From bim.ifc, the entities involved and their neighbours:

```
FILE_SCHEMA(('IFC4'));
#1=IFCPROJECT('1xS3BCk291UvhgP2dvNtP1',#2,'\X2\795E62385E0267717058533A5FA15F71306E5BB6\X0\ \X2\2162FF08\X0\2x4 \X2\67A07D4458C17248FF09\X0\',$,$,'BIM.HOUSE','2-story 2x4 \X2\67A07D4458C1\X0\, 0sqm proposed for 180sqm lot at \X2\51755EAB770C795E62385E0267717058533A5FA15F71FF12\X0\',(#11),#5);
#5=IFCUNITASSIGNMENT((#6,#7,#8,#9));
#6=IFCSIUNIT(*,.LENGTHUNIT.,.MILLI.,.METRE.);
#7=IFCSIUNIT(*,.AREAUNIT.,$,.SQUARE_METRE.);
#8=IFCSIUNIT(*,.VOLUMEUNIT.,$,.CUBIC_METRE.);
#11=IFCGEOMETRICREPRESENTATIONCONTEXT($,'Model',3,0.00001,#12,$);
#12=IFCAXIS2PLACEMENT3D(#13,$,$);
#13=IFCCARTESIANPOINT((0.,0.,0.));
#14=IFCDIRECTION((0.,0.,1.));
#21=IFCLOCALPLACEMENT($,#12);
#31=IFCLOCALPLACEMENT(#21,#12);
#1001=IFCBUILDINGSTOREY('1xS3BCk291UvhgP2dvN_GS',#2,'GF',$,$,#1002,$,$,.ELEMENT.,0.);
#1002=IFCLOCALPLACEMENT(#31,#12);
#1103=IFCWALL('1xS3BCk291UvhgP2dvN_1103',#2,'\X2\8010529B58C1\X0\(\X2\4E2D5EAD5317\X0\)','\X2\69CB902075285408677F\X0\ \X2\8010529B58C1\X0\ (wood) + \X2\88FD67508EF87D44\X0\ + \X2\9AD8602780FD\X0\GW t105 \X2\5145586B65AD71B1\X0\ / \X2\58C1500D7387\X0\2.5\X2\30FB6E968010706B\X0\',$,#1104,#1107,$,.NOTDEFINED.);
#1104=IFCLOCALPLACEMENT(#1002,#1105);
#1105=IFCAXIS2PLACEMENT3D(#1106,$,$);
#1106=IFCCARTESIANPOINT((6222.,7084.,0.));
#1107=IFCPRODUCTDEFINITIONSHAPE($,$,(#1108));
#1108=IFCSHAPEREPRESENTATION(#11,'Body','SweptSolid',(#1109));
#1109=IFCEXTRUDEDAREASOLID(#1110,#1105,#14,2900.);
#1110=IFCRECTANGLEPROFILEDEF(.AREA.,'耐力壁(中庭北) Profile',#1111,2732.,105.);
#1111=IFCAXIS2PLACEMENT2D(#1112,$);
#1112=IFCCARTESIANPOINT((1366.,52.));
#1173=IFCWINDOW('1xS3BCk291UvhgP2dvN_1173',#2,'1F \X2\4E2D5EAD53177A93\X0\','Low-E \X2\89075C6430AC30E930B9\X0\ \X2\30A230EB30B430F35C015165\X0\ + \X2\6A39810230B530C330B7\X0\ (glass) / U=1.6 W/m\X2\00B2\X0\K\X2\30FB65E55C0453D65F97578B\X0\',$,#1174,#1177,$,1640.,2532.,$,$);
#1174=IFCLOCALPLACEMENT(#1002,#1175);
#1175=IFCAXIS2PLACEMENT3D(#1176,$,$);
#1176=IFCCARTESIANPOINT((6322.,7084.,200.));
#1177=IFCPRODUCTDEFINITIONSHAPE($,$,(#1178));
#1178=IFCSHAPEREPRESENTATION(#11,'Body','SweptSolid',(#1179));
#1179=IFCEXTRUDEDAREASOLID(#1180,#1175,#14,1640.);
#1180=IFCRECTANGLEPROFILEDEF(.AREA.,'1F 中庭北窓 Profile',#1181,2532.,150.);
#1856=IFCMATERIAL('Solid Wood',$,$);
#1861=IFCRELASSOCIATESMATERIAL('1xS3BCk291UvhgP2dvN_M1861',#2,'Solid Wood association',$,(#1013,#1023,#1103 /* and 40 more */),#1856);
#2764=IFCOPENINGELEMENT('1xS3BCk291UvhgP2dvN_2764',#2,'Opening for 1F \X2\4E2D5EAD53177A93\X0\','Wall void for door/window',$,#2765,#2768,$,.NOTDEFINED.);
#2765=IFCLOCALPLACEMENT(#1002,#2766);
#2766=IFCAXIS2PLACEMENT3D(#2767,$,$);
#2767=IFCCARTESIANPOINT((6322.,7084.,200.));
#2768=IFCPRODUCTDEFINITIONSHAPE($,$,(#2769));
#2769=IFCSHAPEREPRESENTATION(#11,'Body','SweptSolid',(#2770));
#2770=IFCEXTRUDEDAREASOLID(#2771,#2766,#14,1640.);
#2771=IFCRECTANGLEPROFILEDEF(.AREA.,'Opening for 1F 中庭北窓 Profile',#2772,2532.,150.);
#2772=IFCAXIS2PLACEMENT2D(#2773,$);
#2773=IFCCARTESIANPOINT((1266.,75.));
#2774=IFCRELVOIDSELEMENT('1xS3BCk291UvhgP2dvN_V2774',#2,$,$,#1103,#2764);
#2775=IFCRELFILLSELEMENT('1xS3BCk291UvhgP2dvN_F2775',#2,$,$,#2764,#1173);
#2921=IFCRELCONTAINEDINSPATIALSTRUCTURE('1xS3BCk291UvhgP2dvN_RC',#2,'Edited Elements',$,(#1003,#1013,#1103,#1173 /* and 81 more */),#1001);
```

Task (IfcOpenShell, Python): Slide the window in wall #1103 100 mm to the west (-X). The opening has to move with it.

```python
import ifcopenshell
import ifcopenshell.api.geometry
import ifcopenshell.util.placement

model = ifcopenshell.open("bim.ifc")

window = model.by_guid("1xS3BCk291UvhgP2dvN_1173")
opening = window.FillsVoids[0].RelatingOpeningElement
wall = opening.VoidsElements[0].RelatingBuildingElement

wall_matrix = ifcopenshell.util.placement.get_local_placement(wall.ObjectPlacement)
shift = wall_matrix[:3, 0] * -100.0
before = ifcopenshell.util.placement.get_local_placement(window.ObjectPlacement)[:3, 3].copy()

# The window is not placed relative to its opening, so move both.
for product in (opening, window):
    matrix = ifcopenshell.util.placement.get_local_placement(product.ObjectPlacement)
    matrix[:3, 3] += shift
    ifcopenshell.api.geometry.edit_object_placement(model, product=product, matrix=matrix, is_si=False)

after = ifcopenshell.util.placement.get_local_placement(window.ObjectPlacement)[:3, 3]
print("window moved by", (after - before).round(3) + 0.0)

model.write("bim_rev.ifc")
```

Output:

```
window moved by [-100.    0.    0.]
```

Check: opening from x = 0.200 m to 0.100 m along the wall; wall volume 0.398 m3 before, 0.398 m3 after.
